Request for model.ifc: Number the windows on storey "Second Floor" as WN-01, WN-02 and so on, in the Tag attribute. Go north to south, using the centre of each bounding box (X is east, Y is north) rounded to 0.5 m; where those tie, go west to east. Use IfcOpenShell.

First a look at what the model holds.

```python
import ifcopenshell
import ifcopenshell.util.element
import ifcopenshell.util.placement

model = ifcopenshell.open("model.ifc")
print(model.schema)
storey = next(s for s in model.by_type("IfcBuildingStorey") if s.Name == "Second Floor")
windows = [e for e in ifcopenshell.util.element.get_decomposition(storey) if e.is_a("IfcWindow")]
for e in sorted(windows, key=lambda e: e.id()):
    origin = ifcopenshell.util.placement.get_local_placement(e.ObjectPlacement)[:3, 3]
    print(e.id(), e.Tag, e.Name, origin.round(2) + 0.0, sep=" | ")
```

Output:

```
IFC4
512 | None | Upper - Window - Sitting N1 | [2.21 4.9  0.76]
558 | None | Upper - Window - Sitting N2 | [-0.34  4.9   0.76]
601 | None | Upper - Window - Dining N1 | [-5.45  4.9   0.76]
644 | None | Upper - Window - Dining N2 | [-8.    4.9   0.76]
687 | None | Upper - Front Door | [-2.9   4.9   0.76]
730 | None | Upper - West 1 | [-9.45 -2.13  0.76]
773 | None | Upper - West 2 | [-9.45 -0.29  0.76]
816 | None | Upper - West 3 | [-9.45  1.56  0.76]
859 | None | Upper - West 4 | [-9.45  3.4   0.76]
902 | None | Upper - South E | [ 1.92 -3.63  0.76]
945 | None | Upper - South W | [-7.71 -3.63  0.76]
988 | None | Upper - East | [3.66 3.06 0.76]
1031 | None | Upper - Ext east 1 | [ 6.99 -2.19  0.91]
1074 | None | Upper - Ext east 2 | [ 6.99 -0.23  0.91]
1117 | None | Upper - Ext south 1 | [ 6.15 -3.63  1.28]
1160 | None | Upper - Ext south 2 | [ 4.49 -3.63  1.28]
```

```python
import ifcopenshell
import ifcopenshell.geom
import ifcopenshell.util.element
import ifcopenshell.util.shape

model = ifcopenshell.open("model.ifc")
settings = ifcopenshell.geom.settings()
settings.set("use-world-coords", True)


def centre(element):
    shape = ifcopenshell.geom.create_shape(settings, element)
    return ifcopenshell.util.shape.get_bbox_centroid(shape.geometry)


storey = next(s for s in model.by_type("IfcBuildingStorey") if s.Name == "Second Floor")
windows = [e for e in ifcopenshell.util.element.get_decomposition(storey) if e.is_a("IfcWindow")]

# Insertion points can sit at a corner or the storey origin, so sort by the geometry (in metres).
centres = {e: centre(e) for e in windows}
windows.sort(key=lambda e: (-round(centres[e][1] / 0.5), centres[e][0]))

for i, e in enumerate(windows, start=1):
    number = f"WN-{i:02d}"
    e.Tag = number
    print(e.id(), number)

model.write("model_edited.ifc")
```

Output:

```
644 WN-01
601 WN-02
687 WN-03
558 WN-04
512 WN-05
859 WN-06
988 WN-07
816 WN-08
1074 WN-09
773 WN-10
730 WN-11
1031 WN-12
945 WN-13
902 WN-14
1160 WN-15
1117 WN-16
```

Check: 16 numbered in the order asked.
